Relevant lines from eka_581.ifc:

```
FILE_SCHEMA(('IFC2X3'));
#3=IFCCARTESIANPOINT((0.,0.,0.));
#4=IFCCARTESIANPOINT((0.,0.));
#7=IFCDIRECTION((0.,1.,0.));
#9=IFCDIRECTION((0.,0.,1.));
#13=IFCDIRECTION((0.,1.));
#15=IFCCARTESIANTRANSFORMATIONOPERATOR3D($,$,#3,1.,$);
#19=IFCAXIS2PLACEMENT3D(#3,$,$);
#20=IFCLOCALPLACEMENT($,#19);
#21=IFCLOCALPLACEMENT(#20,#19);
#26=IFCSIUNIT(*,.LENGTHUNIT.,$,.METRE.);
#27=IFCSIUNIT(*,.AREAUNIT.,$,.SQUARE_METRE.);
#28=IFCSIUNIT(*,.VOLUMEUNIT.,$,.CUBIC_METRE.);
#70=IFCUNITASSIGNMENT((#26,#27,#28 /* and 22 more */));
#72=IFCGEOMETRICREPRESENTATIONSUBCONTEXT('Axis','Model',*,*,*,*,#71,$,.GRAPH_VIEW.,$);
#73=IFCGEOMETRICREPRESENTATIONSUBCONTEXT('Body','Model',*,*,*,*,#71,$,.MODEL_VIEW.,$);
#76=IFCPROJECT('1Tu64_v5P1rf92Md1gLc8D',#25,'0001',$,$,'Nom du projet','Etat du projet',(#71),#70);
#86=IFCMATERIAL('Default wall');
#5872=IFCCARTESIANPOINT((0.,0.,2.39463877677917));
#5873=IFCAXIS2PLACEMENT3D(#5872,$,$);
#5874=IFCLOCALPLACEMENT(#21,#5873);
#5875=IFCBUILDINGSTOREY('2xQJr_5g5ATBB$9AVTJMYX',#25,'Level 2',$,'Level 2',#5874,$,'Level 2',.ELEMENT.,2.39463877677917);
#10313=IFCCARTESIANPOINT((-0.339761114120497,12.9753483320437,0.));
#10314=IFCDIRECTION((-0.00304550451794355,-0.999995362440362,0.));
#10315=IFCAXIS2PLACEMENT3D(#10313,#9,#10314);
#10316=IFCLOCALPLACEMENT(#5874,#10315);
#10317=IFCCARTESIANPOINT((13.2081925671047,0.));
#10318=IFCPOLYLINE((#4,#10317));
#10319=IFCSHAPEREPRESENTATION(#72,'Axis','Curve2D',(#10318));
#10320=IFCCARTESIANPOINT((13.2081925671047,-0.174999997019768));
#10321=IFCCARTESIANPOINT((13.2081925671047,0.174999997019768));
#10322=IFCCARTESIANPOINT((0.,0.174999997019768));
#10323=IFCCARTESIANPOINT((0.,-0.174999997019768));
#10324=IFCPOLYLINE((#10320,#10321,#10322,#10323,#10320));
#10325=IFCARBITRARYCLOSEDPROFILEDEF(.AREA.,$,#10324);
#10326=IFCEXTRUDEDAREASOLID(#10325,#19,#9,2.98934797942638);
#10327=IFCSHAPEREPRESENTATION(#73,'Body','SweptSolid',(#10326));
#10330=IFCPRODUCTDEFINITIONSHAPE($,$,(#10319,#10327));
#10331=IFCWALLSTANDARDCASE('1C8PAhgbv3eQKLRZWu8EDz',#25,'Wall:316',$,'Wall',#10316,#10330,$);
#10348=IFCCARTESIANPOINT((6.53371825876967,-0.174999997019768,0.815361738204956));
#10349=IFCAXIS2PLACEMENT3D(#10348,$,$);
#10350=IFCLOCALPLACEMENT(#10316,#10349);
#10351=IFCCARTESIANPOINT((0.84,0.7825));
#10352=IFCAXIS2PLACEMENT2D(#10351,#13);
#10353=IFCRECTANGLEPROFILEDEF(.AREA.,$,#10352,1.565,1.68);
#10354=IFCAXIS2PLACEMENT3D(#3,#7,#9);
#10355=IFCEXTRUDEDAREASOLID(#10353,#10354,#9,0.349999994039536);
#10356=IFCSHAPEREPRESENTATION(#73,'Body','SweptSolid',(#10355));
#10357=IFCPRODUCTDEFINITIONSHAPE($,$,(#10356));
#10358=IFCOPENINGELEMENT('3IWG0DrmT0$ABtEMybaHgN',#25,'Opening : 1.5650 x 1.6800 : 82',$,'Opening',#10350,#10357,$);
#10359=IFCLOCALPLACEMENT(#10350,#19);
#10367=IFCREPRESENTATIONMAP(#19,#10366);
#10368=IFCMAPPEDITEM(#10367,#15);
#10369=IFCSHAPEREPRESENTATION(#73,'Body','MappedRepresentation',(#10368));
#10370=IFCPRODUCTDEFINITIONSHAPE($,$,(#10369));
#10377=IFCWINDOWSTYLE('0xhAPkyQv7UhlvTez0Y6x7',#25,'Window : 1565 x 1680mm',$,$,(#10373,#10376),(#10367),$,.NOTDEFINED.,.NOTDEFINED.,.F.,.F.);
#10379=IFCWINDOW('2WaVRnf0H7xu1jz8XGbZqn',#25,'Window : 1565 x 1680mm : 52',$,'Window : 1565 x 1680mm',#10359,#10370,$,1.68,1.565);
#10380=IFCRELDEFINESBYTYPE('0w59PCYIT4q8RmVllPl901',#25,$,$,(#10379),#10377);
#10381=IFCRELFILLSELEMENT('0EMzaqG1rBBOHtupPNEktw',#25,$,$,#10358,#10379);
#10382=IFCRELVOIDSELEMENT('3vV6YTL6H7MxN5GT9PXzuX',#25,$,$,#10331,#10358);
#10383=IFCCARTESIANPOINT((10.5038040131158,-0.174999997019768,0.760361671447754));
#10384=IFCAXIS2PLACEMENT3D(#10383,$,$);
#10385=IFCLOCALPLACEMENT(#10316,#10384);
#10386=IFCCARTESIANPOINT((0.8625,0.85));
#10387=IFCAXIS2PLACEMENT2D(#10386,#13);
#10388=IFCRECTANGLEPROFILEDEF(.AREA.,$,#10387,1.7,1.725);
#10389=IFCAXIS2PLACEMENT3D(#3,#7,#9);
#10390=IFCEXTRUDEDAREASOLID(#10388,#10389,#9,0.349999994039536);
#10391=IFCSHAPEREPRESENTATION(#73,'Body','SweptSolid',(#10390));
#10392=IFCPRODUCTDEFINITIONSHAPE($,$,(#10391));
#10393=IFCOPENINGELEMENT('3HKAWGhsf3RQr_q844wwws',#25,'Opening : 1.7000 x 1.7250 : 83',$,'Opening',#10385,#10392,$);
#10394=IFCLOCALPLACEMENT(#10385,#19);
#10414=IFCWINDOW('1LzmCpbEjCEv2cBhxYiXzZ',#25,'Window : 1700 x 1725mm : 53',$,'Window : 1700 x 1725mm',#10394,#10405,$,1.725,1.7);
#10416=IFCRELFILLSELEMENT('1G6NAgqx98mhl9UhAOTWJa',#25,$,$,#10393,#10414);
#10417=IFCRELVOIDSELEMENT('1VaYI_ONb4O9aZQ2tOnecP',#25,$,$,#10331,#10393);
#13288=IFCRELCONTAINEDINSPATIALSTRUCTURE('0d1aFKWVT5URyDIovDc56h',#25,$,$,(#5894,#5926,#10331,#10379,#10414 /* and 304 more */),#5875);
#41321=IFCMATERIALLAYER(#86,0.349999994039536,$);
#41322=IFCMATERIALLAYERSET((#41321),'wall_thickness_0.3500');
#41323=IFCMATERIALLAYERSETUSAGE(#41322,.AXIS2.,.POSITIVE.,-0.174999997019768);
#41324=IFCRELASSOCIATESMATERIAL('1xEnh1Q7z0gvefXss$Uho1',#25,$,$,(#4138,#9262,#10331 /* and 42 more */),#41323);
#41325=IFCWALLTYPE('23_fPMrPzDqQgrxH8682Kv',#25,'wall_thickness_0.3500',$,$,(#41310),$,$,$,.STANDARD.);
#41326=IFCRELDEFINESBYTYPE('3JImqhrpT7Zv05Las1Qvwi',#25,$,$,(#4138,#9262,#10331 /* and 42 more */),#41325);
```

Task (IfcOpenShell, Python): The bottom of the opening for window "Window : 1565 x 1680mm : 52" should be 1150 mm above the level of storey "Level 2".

```python
import numpy as np
import ifcopenshell
import ifcopenshell.api.geometry
import ifcopenshell.geom
import ifcopenshell.util.element
import ifcopenshell.util.placement
import ifcopenshell.util.shape
import ifcopenshell.util.unit

model = ifcopenshell.open("eka_581.ifc")
unit_scale = ifcopenshell.util.unit.calculate_unit_scale(model)

window = model.by_id(10379)
opening = window.FillsVoids[0].RelatingOpeningElement
storey = ifcopenshell.util.element.get_container(window, ifc_class="IfcBuildingStorey")
level = ifcopenshell.util.placement.get_local_placement(storey.ObjectPlacement)[2, 3]

# The opening's origin need not be at the sill, so measure its lowest point.
shape = ifcopenshell.geom.create_shape(ifcopenshell.geom.settings(), opening)
bottom = ifcopenshell.util.shape.get_shape_bottom_elevation(shape, shape.geometry) / unit_scale
dz = level + 1.15 / unit_scale - bottom

shift = np.array([0.0, 0.0, dz])
# The window is placed relative to its opening, so it follows when the opening moves.
matrix = ifcopenshell.util.placement.get_local_placement(opening.ObjectPlacement)
matrix[:3, 3] += shift
ifcopenshell.api.geometry.edit_object_placement(
    model, product=opening, matrix=matrix, is_si=False, should_transform_children=True
)

print(f"moved by {dz * unit_scale:+.3f} m")

model.write("eka_581-out.ifc")
```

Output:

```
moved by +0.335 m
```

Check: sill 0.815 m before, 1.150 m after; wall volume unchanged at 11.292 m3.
